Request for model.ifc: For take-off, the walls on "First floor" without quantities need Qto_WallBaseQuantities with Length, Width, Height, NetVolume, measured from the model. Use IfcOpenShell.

First a look at what the model holds.

```python
import ifcopenshell
import ifcopenshell.util.element
import ifcopenshell.util.unit

model = ifcopenshell.open("model.ifc")
print(model.schema)
for unit_type in ("LENGTHUNIT", "AREAUNIT", "VOLUMEUNIT"):
    print(unit_type, ifcopenshell.util.unit.calculate_unit_scale(model, unit_type))
storey = next(s for s in model.by_type("IfcBuildingStorey") if s.Name == "First floor")
walls = [e for e in ifcopenshell.util.element.get_decomposition(storey) if e.is_a("IfcWall")]
for e in sorted(walls, key=lambda e: e.id()):
    print(e.id(), e.is_a(), e.Name, list(ifcopenshell.util.element.get_psets(e, qtos_only=True)), sep=" | ")
```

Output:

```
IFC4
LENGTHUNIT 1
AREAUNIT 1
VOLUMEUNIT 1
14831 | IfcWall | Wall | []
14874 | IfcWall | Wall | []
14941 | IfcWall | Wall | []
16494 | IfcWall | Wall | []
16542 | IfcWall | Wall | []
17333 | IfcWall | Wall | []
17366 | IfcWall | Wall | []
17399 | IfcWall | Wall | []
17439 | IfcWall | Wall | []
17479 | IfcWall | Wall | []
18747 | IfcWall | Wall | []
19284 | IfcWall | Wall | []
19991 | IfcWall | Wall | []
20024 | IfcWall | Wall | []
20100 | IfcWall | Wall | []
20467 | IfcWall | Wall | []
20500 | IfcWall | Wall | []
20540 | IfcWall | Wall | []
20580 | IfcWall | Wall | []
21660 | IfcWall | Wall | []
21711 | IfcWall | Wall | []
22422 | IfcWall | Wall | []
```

```python
import ifcopenshell
import ifcopenshell.api.pset
import ifcopenshell.geom
import ifcopenshell.util.element
import ifcopenshell.util.shape
import ifcopenshell.util.unit

model = ifcopenshell.open("model.ifc")
unit_scale = ifcopenshell.util.unit.calculate_unit_scale(model)
volume_scale = ifcopenshell.util.unit.calculate_unit_scale(model, "VOLUMEUNIT")
settings = ifcopenshell.geom.settings()

storey = next(s for s in model.by_type("IfcBuildingStorey") if s.Name == "First floor")
walls = [e for e in ifcopenshell.util.element.get_decomposition(storey) if e.is_a("IfcWall")]

for e in sorted(walls, key=lambda e: e.id()):
    if ifcopenshell.util.element.get_psets(e, qtos_only=True, should_inherit=False):
        continue
    # Geometry comes back in metres, in the element's own axes.
    shape = ifcopenshell.geom.create_shape(settings, e)
    values = {
        "Length": ifcopenshell.util.shape.get_x(shape.geometry) / unit_scale,
        "Width": ifcopenshell.util.shape.get_y(shape.geometry) / unit_scale,
        "Height": ifcopenshell.util.shape.get_z(shape.geometry) / unit_scale,
        "NetVolume": ifcopenshell.util.shape.get_volume(shape.geometry) / volume_scale,
    }
    qto = ifcopenshell.api.pset.add_qto(model, product=e, name="Qto_WallBaseQuantities")
    ifcopenshell.api.pset.edit_qto(model, qto=qto, properties=values)
    print(e.id(), {k: round(v, 3) for k, v in values.items()})

model.write("model_edited.ifc")
```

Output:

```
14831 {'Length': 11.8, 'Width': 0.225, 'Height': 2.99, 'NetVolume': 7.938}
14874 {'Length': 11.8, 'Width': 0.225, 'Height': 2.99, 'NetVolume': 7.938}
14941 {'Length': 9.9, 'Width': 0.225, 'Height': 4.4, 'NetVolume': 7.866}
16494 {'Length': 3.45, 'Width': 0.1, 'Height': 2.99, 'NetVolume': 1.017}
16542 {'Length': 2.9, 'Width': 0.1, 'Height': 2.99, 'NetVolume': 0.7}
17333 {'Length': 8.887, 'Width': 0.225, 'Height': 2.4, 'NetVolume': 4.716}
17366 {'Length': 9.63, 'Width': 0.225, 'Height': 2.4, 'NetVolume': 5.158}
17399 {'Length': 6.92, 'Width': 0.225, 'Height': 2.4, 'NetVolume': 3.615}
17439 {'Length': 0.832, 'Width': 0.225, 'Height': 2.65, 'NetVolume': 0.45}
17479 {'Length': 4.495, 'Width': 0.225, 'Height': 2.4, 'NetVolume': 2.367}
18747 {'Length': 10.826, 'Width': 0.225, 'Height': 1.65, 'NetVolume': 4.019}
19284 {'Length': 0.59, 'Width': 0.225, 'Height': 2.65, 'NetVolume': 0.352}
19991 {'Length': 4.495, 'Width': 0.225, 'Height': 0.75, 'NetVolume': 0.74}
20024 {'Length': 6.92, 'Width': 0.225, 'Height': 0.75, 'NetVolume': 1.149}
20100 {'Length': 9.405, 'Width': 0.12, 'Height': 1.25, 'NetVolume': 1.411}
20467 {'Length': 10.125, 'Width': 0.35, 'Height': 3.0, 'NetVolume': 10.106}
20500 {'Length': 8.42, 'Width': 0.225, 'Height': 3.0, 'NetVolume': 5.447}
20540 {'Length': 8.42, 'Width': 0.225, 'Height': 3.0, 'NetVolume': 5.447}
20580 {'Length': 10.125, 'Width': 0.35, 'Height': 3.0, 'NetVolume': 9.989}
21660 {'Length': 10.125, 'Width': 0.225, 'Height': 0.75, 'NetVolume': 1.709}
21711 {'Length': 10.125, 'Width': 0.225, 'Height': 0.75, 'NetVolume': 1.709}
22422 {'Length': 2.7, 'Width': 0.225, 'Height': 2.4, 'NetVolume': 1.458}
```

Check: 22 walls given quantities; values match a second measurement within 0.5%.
